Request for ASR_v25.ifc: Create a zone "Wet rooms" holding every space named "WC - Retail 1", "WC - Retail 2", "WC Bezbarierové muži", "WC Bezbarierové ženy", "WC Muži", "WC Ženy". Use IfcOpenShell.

First a look at what the model holds.

```python
import ifcopenshell

model = ifcopenshell.open("ASR_v25.ifc")
print(model.schema)
seen = {}
for space in model.by_type("IfcSpace"):
    seen[space.LongName] = seen.get(space.LongName, 0) + 1
for name, count in sorted(seen.items(), key=str):
    print(count, "x", name)
print("zones:", [z.Name for z in model.by_type("IfcZone")][:20])
```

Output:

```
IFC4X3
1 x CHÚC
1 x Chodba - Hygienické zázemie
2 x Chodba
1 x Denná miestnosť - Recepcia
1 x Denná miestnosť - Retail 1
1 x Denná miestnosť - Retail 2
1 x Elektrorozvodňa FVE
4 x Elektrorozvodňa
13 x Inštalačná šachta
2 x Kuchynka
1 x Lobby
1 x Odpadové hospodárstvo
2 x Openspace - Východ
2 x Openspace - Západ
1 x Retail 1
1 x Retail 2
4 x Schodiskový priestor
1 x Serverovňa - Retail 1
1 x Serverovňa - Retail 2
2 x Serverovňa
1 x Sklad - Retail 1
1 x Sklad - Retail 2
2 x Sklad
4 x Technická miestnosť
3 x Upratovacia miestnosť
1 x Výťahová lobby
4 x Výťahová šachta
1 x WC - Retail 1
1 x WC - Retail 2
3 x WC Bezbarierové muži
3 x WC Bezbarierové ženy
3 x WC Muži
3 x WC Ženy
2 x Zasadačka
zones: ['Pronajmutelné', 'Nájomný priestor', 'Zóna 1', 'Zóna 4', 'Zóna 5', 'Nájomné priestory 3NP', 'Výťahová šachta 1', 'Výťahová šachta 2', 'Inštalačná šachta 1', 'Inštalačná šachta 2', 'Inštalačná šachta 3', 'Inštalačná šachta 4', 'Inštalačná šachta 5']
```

```python
import ifcopenshell
import ifcopenshell.api.group
import ifcopenshell.api.root

model = ifcopenshell.open("ASR_v25.ifc")

names = {"WC - Retail 1", "WC - Retail 2", "WC Bezbarierové muži", "WC Bezbarierové ženy", "WC Muži", "WC Ženy"}
spaces = [s for s in model.by_type("IfcSpace") if s.LongName in names]

zone = ifcopenshell.api.root.create_entity(model, ifc_class="IfcZone", name="Wet rooms")
ifcopenshell.api.group.assign_group(model, products=spaces, group=zone)
print(len(spaces), "spaces in", zone.Name)

model.write("ASR_v25-out.ifc")
```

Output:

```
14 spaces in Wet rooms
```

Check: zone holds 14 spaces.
